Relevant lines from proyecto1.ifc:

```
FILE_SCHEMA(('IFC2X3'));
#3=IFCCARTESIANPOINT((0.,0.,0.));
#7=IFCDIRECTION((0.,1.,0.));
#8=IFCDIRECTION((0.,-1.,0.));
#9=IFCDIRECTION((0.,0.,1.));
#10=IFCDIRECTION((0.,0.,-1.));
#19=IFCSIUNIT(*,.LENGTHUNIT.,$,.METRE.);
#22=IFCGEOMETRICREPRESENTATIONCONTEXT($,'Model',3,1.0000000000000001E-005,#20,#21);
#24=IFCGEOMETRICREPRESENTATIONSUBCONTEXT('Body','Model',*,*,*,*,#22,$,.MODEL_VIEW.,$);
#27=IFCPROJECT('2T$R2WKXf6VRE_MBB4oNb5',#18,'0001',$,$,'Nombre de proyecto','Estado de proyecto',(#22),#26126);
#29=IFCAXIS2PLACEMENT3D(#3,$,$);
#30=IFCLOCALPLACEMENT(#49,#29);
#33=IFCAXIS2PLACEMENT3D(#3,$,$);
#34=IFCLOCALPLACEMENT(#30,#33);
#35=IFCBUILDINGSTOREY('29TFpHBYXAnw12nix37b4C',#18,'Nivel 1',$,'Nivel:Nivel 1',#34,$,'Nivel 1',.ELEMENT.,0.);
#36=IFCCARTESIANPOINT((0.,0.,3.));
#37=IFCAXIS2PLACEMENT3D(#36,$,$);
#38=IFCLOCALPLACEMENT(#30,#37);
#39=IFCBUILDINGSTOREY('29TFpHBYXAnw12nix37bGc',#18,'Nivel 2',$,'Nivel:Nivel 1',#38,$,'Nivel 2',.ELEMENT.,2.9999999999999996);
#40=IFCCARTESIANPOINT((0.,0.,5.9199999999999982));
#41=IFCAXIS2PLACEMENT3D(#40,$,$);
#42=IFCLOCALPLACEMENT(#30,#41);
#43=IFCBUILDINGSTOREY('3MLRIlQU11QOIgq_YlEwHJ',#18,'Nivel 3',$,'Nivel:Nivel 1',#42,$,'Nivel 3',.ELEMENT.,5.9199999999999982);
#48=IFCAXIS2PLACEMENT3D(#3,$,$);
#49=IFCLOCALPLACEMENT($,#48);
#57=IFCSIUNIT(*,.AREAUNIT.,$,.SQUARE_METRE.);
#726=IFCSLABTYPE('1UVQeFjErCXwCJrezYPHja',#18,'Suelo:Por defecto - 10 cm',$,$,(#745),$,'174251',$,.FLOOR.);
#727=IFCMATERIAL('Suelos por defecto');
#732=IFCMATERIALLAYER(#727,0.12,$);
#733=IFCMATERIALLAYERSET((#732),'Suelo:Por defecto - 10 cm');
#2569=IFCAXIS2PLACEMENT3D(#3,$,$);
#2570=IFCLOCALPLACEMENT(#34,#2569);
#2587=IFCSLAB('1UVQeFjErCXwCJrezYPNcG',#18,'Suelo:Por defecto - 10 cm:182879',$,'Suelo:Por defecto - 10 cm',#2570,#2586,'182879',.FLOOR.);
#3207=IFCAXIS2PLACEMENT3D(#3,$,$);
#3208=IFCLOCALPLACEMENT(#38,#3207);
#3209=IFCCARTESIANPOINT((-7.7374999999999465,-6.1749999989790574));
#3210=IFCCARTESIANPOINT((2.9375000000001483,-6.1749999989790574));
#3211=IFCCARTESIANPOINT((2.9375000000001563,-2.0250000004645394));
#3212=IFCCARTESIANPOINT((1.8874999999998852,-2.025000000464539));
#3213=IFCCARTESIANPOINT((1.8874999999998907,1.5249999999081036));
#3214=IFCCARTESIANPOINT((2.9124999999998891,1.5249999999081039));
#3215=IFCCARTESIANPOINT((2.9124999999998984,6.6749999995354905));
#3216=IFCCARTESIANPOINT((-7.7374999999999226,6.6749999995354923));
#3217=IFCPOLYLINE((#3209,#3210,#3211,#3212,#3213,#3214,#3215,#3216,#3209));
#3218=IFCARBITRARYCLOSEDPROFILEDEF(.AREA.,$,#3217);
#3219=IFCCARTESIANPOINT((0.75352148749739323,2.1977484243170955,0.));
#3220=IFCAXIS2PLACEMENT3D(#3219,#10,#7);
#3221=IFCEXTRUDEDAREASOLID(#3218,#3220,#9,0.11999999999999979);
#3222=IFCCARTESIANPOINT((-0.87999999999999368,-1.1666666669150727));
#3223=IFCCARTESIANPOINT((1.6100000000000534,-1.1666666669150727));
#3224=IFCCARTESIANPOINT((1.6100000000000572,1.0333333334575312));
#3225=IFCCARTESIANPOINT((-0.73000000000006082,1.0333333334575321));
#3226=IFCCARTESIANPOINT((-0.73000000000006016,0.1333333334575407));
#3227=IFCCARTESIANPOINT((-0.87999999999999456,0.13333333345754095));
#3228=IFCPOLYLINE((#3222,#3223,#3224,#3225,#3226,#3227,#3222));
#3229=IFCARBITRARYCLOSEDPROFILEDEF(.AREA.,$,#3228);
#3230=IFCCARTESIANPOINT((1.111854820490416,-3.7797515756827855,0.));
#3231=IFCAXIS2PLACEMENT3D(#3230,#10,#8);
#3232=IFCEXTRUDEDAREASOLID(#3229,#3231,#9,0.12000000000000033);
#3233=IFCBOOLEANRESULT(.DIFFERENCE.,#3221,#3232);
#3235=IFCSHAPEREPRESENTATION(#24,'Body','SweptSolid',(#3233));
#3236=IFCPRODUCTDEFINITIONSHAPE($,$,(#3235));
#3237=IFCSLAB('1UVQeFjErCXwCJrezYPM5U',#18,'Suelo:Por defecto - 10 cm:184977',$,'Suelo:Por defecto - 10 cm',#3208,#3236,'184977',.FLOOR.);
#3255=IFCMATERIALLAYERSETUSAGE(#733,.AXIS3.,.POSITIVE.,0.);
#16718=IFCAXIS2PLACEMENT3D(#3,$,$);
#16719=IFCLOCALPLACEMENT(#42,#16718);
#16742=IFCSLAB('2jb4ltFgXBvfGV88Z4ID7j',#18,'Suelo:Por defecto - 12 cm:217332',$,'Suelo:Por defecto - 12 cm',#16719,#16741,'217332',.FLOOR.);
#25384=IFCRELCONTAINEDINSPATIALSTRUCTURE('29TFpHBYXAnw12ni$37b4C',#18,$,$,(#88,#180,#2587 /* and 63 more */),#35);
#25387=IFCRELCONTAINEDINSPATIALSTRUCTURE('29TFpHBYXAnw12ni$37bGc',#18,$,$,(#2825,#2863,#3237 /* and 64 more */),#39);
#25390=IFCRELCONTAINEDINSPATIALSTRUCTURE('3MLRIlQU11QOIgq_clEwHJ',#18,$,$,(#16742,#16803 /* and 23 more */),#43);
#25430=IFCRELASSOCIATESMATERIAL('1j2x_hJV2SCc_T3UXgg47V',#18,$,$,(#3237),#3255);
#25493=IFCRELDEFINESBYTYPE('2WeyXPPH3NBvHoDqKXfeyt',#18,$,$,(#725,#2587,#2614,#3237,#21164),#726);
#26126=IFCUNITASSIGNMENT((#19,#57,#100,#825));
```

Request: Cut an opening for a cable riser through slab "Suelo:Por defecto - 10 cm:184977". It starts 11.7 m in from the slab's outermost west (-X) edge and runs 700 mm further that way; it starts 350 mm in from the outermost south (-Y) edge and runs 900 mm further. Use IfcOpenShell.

```python
import numpy as np
import ifcopenshell
import ifcopenshell.api.feature
import ifcopenshell.api.geometry
import ifcopenshell.api.root
import ifcopenshell.geom
import ifcopenshell.util.placement
import ifcopenshell.util.representation
import ifcopenshell.util.shape
import ifcopenshell.util.unit

model = ifcopenshell.open("proyecto1.ifc")
unit_scale = ifcopenshell.util.unit.calculate_unit_scale(model)
settings = ifcopenshell.geom.settings()


def volume(element):
    """Net volume in cubic metres, openings subtracted."""
    shape = ifcopenshell.geom.create_shape(settings, element)
    return ifcopenshell.util.shape.get_volume(shape.geometry)


slab = model.by_id(3237)
before = volume(slab)

# Extent in the slab's own axes, in metres. The edges named are its -X and -Y sides.
slab_shape = ifcopenshell.geom.create_shape(settings, slab)
vertices = ifcopenshell.util.shape.get_vertices(slab_shape.geometry)
x_min, y_min, bottom = vertices.min(axis=0)
top = vertices[:, 2].max()

opening = ifcopenshell.api.root.create_entity(model, ifc_class="IfcOpeningElement", name="Cable riser opening")
context = ifcopenshell.util.representation.get_context(model, "Model", "Body", "MODEL_VIEW")
width, depth = 0.7, 0.9
outline = [(0.0, 0.0), (width, 0.0), (width, depth), (0.0, depth), (0.0, 0.0)]
# Overshoot both faces by 50 mm so the cut is clean.
shape = ifcopenshell.api.geometry.add_slab_representation(
    model, context=context, depth=top - bottom + 0.1, polyline=outline
)
ifcopenshell.api.geometry.assign_representation(model, product=opening, representation=shape)

matrix = ifcopenshell.util.placement.get_local_placement(slab.ObjectPlacement)
matrix[:, 3] = matrix @ np.append(np.array([x_min + 11.7, y_min + 0.35, bottom - 0.05]) / unit_scale, 1.0)
ifcopenshell.api.geometry.edit_object_placement(model, product=opening, matrix=matrix, is_si=False)
ifcopenshell.api.feature.add_feature(model, feature=opening, element=slab)

after = volume(slab)

print(f"slab volume {before:.3f} -> {after:.3f} m3")

model.write("proyecto1-out.ifc")
```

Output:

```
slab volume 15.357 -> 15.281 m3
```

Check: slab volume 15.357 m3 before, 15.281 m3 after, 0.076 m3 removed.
